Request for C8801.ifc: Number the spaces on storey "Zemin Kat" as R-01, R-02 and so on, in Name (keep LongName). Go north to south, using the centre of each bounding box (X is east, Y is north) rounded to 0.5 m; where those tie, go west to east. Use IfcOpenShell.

First a look at what the model holds.

```python
import ifcopenshell
import ifcopenshell.util.element
import ifcopenshell.util.placement

model = ifcopenshell.open("C8801.ifc")
print(model.schema)
storey = next(s for s in model.by_type("IfcBuildingStorey") if s.Name == "Zemin Kat")
spaces = [e for e in ifcopenshell.util.element.get_decomposition(storey) if e.is_a("IfcSpace")]
for e in sorted(spaces, key=lambda e: e.id()):
    origin = ifcopenshell.util.placement.get_local_placement(e.ObjectPlacement)[:3, 3]
    print(e.id(), e.Name, e.LongName, origin.round(2) + 0.0, sep=" | ")
```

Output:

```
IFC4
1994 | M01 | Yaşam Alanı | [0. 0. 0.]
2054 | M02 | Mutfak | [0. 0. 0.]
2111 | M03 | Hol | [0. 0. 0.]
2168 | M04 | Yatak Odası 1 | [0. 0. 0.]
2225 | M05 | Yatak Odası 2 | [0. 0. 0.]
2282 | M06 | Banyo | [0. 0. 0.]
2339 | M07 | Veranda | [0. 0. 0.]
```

```python
import ifcopenshell
import ifcopenshell.geom
import ifcopenshell.util.element
import ifcopenshell.util.shape

model = ifcopenshell.open("C8801.ifc")
settings = ifcopenshell.geom.settings()
settings.set("use-world-coords", True)


def centre(element):
    shape = ifcopenshell.geom.create_shape(settings, element)
    return ifcopenshell.util.shape.get_bbox_centroid(shape.geometry)


storey = next(s for s in model.by_type("IfcBuildingStorey") if s.Name == "Zemin Kat")
spaces = [e for e in ifcopenshell.util.element.get_decomposition(storey) if e.is_a("IfcSpace")]

# Insertion points can sit at a corner or the storey origin, so sort by the geometry (in metres).
centres = {e: centre(e) for e in spaces}
spaces.sort(key=lambda e: (-round(centres[e][1] / 0.5), centres[e][0]))

for i, e in enumerate(spaces, start=1):
    number = f"R-{i:02d}"
    e.Name = number
    print(e.id(), number)

model.write("C8801_v2.ifc")
```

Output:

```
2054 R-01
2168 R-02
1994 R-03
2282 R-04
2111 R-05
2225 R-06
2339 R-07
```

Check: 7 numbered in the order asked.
